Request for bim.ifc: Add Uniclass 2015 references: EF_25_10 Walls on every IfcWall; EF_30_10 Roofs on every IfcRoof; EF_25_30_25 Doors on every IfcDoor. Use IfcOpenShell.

First a look at what the model holds.

```python
import ifcopenshell

model = ifcopenshell.open("bim.ifc")
print(model.schema)
print("classifications:", [c.Name for c in model.by_type("IfcClassification")])
for ifc_class in ("IfcDoor", "IfcRoof", "IfcStair", "IfcWall", "IfcWindow"):
    print(ifc_class, len(model.by_type(ifc_class)))
```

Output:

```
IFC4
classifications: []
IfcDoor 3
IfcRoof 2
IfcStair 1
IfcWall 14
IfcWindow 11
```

```python
import ifcopenshell
import ifcopenshell.api.classification

model = ifcopenshell.open("bim.ifc")

system = ifcopenshell.api.classification.add_classification(model, classification="Uniclass 2015")

codes = {
    "IfcWall": ("EF_25_10", "Walls"),
    "IfcRoof": ("EF_30_10", "Roofs"),
    "IfcDoor": ("EF_25_30_25", "Doors"),
}
for ifc_class, (code, name) in codes.items():
    products = model.by_type(ifc_class)
    ifcopenshell.api.classification.add_reference(
        model, products=products, classification=system, identification=code, name=name
    )
    print(code, len(products))

model.write("bim_v2.ifc")
```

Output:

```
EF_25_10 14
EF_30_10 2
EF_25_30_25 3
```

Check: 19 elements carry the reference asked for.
